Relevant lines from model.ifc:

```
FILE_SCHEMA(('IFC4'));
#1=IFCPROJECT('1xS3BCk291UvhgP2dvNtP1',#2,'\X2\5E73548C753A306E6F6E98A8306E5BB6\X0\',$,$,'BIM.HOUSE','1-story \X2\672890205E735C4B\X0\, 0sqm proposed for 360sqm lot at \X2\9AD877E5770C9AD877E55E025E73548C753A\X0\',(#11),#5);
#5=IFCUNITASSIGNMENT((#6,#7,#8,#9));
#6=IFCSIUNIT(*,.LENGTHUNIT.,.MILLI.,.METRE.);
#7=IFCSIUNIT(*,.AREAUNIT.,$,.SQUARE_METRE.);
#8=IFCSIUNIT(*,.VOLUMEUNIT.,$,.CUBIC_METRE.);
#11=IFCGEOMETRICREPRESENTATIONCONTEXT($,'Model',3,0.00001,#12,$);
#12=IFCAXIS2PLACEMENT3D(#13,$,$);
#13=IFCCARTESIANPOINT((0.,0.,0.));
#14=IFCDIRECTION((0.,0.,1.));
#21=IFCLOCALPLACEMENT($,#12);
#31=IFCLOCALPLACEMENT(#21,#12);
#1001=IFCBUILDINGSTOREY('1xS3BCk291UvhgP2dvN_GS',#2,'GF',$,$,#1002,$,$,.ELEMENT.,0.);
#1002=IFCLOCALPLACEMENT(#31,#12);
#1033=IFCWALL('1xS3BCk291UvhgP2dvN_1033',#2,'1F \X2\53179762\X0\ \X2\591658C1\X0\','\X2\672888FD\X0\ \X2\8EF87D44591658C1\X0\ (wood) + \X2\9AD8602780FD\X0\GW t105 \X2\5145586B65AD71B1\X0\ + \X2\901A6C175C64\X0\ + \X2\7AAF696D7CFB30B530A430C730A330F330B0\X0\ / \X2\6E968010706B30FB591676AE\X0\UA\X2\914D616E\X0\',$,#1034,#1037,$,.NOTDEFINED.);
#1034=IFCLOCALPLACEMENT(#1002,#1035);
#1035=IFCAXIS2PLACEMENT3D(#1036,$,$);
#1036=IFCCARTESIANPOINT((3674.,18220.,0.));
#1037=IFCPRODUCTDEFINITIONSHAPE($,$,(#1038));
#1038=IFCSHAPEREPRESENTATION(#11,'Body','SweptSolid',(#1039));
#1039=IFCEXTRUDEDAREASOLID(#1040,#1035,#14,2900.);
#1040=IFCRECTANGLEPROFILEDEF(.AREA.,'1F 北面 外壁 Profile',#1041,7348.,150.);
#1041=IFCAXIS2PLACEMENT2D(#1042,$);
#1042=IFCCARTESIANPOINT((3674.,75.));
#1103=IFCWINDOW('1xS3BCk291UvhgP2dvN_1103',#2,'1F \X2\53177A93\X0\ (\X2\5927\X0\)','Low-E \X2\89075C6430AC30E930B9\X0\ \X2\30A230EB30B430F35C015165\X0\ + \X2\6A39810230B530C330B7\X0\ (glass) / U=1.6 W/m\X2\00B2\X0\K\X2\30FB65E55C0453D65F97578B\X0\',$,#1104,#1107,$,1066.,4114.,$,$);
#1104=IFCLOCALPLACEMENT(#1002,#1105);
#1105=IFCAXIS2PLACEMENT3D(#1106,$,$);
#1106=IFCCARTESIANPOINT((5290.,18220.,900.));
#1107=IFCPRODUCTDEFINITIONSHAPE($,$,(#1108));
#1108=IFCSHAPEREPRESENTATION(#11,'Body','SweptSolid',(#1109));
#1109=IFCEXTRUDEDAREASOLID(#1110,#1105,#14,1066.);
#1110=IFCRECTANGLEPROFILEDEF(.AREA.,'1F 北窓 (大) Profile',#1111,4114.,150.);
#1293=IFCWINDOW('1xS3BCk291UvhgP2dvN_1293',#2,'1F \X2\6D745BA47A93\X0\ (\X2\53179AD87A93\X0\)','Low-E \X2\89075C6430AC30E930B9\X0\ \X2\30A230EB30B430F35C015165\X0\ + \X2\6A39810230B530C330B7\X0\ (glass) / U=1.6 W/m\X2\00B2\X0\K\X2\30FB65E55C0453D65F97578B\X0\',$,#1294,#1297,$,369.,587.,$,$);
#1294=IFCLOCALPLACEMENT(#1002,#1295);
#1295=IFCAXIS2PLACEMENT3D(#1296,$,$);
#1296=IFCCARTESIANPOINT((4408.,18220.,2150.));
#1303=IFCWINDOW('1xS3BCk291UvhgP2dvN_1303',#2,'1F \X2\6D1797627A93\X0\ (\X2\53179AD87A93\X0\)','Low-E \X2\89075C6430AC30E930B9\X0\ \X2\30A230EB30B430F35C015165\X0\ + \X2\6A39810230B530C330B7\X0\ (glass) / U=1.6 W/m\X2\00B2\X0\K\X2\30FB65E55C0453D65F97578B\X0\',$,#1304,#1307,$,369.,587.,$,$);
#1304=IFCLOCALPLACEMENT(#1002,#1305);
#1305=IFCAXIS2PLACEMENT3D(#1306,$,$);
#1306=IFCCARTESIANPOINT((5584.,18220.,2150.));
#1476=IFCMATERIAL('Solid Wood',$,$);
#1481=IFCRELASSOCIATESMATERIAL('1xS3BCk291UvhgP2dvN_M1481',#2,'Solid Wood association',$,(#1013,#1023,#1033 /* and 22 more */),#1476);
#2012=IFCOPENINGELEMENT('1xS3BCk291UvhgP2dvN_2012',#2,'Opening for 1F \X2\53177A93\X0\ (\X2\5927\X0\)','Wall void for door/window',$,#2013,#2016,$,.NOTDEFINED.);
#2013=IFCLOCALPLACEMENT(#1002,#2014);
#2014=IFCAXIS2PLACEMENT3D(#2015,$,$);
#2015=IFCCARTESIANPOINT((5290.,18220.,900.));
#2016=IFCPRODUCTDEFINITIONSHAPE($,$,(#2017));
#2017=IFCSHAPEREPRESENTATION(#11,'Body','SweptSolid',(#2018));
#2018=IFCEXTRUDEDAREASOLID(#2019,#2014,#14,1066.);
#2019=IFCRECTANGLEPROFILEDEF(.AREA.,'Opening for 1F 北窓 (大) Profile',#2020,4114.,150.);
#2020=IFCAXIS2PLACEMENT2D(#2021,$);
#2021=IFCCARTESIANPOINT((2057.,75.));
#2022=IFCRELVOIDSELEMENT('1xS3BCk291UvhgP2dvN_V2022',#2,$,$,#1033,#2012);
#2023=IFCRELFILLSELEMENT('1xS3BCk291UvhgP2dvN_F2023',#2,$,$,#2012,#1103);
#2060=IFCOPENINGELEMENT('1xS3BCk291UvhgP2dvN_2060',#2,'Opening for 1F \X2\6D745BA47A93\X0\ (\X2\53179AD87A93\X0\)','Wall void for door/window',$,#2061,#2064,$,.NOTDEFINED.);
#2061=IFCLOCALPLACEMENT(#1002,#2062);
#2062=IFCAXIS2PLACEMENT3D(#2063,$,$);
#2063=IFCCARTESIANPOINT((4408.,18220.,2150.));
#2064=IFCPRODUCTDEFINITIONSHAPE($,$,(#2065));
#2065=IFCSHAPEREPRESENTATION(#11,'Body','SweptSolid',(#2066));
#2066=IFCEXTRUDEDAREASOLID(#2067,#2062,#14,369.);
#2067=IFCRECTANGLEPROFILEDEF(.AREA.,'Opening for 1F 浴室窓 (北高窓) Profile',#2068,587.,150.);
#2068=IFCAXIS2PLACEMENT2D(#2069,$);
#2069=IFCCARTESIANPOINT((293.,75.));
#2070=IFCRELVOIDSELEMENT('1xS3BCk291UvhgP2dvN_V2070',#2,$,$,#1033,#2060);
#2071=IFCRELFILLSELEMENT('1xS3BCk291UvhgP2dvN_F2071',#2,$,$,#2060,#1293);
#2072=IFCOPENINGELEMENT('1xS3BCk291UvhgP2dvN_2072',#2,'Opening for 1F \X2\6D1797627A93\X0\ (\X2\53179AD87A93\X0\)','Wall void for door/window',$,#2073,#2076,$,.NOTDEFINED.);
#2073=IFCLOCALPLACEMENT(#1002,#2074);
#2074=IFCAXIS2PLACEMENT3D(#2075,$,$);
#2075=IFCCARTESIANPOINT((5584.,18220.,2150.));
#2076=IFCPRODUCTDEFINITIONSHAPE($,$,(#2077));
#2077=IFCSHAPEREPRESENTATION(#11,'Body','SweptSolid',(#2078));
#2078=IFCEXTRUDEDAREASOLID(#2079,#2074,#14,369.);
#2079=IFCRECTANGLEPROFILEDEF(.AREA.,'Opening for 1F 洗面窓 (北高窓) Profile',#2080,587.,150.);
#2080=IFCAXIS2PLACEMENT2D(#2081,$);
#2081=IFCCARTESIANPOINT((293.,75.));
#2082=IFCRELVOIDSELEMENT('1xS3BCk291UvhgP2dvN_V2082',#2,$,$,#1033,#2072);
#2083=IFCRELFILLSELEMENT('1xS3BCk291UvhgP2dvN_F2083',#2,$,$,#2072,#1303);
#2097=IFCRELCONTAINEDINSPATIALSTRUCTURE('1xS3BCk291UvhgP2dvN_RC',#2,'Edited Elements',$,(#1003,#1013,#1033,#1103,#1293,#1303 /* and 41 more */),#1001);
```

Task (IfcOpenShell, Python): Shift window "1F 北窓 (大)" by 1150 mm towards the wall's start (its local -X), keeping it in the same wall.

```python
import ifcopenshell
import ifcopenshell.api.geometry
import ifcopenshell.util.placement

model = ifcopenshell.open("model.ifc")

window = model.by_guid("1xS3BCk291UvhgP2dvN_1103")
opening = window.FillsVoids[0].RelatingOpeningElement
wall = opening.VoidsElements[0].RelatingBuildingElement

wall_matrix = ifcopenshell.util.placement.get_local_placement(wall.ObjectPlacement)
shift = wall_matrix[:3, 0] * -1150.0
before = ifcopenshell.util.placement.get_local_placement(window.ObjectPlacement)[:3, 3].copy()

# The window is not placed relative to its opening, so move both.
for product in (opening, window):
    matrix = ifcopenshell.util.placement.get_local_placement(product.ObjectPlacement)
    matrix[:3, 3] += shift
    ifcopenshell.api.geometry.edit_object_placement(model, product=product, matrix=matrix, is_si=False)

after = ifcopenshell.util.placement.get_local_placement(window.ObjectPlacement)[:3, 3]
print("window moved by", (after - before).round(3) + 0.0)

model.write("model_v2.ifc")
```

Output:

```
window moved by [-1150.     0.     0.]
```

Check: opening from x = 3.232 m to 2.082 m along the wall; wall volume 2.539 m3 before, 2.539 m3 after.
